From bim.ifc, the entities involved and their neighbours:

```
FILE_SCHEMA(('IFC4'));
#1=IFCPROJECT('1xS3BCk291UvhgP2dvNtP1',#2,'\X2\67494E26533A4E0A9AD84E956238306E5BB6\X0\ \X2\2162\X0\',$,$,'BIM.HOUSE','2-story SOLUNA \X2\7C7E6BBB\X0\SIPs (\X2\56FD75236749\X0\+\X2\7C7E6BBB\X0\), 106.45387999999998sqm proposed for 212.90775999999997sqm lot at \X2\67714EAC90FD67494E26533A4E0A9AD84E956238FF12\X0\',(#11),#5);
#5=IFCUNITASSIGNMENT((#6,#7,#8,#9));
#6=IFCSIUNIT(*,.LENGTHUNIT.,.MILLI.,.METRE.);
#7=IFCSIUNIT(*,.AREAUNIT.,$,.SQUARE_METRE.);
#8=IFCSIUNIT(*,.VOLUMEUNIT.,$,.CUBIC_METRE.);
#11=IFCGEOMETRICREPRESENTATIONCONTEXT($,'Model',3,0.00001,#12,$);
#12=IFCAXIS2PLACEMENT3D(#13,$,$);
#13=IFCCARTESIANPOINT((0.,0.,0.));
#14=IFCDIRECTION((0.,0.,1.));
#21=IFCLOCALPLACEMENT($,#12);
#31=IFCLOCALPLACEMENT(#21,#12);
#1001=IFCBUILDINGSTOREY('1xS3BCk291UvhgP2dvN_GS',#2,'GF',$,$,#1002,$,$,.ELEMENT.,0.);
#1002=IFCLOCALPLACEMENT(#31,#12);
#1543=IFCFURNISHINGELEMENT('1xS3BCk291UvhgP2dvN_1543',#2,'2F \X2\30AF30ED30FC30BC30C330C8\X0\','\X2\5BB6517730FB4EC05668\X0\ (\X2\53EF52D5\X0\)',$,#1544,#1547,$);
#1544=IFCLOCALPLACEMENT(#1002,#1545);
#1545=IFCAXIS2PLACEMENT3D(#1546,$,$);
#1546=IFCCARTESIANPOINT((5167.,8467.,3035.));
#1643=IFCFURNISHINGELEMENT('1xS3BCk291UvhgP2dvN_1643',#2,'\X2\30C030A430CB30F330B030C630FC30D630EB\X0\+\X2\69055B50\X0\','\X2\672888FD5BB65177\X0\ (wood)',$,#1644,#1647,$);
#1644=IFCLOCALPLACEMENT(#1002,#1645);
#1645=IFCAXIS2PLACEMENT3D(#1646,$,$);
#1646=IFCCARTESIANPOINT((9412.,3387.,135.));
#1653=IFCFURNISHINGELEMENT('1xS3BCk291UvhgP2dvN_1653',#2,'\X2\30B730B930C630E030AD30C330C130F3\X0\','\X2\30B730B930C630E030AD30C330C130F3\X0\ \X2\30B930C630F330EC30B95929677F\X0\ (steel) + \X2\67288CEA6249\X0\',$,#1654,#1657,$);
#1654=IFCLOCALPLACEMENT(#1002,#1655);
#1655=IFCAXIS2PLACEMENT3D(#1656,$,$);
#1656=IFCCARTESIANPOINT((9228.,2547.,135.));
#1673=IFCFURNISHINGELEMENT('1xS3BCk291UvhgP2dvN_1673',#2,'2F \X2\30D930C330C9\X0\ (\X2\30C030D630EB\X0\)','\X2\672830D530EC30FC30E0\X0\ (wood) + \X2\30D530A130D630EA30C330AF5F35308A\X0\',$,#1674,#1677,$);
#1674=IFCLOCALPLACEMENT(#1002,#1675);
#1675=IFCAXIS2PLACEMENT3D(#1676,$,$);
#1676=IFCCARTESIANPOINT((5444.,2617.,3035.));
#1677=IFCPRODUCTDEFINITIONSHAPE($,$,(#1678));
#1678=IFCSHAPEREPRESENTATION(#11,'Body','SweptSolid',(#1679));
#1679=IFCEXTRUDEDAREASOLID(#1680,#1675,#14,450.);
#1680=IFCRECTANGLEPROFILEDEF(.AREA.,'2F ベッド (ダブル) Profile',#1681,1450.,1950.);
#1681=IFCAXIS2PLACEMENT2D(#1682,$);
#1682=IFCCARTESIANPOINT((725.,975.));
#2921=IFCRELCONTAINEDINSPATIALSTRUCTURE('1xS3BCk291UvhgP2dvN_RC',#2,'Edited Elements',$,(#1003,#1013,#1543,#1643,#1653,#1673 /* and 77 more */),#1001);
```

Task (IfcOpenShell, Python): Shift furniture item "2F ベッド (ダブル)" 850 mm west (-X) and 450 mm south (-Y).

```python
import ifcopenshell
import ifcopenshell.api.geometry
import ifcopenshell.util.placement

model = ifcopenshell.open("bim.ifc")

item = model.by_id(1673)
matrix = ifcopenshell.util.placement.get_local_placement(item.ObjectPlacement)
matrix[0, 3] -= 850.0
matrix[1, 3] -= 450.0
ifcopenshell.api.geometry.edit_object_placement(model, product=item, matrix=matrix, is_si=False)

print(ifcopenshell.util.placement.get_local_placement(item.ObjectPlacement).round(3) + 0.0)

model.write("bim_v2.ifc")
```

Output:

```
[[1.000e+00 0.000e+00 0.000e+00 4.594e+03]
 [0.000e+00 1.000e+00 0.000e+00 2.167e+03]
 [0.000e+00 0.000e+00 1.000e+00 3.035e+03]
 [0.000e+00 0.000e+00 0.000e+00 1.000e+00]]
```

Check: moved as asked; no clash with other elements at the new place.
